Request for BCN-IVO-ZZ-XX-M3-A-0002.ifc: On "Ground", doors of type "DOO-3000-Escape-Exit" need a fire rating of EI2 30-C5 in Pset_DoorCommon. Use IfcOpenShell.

First a look at what the model holds.

```python
import ifcopenshell
import ifcopenshell.util.element

model = ifcopenshell.open("BCN-IVO-ZZ-XX-M3-A-0002.ifc")
print(model.schema)
storey = next(s for s in model.by_type("IfcBuildingStorey") if s.Name == "Ground")
doors = [e for e in ifcopenshell.util.element.get_decomposition(storey) if e.is_a("IfcDoor")]
seen = {}
for e in doors:
    element_type = ifcopenshell.util.element.get_type(e)
    key = (element_type.Name if element_type != e and element_type else None, ifcopenshell.util.element.get_pset(e, "Pset_DoorCommon", "FireRating"))
    seen[key] = seen.get(key, 0) + 1
for (name, value), count in sorted(seen.items(), key=str):
    print(count, "x", name, "|", value)
```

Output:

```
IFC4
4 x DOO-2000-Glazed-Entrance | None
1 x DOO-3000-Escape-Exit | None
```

```python
import ifcopenshell
import ifcopenshell.api.pset
import ifcopenshell.util.element

model = ifcopenshell.open("BCN-IVO-ZZ-XX-M3-A-0002.ifc")

storey = next(s for s in model.by_type("IfcBuildingStorey") if s.Name == "Ground")
doors = [e for e in ifcopenshell.util.element.get_decomposition(storey) if e.is_a("IfcDoor")]

count = 0
for e in doors:
    element_type = ifcopenshell.util.element.get_type(e)
    if element_type in (None, e) or element_type.Name != "DOO-3000-Escape-Exit":
        continue
    # add_pset returns the element's existing set when there is one.
    pset = ifcopenshell.api.pset.add_pset(model, product=e, name="Pset_DoorCommon")
    ifcopenshell.api.pset.edit_pset(model, pset=pset, properties={"FireRating": "EI2 30-C5"})
    count += 1

print(count, "doors updated")

model.write("BCN-IVO-ZZ-XX-M3-A-0002-out.ifc")
```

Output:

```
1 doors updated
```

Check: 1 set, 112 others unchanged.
